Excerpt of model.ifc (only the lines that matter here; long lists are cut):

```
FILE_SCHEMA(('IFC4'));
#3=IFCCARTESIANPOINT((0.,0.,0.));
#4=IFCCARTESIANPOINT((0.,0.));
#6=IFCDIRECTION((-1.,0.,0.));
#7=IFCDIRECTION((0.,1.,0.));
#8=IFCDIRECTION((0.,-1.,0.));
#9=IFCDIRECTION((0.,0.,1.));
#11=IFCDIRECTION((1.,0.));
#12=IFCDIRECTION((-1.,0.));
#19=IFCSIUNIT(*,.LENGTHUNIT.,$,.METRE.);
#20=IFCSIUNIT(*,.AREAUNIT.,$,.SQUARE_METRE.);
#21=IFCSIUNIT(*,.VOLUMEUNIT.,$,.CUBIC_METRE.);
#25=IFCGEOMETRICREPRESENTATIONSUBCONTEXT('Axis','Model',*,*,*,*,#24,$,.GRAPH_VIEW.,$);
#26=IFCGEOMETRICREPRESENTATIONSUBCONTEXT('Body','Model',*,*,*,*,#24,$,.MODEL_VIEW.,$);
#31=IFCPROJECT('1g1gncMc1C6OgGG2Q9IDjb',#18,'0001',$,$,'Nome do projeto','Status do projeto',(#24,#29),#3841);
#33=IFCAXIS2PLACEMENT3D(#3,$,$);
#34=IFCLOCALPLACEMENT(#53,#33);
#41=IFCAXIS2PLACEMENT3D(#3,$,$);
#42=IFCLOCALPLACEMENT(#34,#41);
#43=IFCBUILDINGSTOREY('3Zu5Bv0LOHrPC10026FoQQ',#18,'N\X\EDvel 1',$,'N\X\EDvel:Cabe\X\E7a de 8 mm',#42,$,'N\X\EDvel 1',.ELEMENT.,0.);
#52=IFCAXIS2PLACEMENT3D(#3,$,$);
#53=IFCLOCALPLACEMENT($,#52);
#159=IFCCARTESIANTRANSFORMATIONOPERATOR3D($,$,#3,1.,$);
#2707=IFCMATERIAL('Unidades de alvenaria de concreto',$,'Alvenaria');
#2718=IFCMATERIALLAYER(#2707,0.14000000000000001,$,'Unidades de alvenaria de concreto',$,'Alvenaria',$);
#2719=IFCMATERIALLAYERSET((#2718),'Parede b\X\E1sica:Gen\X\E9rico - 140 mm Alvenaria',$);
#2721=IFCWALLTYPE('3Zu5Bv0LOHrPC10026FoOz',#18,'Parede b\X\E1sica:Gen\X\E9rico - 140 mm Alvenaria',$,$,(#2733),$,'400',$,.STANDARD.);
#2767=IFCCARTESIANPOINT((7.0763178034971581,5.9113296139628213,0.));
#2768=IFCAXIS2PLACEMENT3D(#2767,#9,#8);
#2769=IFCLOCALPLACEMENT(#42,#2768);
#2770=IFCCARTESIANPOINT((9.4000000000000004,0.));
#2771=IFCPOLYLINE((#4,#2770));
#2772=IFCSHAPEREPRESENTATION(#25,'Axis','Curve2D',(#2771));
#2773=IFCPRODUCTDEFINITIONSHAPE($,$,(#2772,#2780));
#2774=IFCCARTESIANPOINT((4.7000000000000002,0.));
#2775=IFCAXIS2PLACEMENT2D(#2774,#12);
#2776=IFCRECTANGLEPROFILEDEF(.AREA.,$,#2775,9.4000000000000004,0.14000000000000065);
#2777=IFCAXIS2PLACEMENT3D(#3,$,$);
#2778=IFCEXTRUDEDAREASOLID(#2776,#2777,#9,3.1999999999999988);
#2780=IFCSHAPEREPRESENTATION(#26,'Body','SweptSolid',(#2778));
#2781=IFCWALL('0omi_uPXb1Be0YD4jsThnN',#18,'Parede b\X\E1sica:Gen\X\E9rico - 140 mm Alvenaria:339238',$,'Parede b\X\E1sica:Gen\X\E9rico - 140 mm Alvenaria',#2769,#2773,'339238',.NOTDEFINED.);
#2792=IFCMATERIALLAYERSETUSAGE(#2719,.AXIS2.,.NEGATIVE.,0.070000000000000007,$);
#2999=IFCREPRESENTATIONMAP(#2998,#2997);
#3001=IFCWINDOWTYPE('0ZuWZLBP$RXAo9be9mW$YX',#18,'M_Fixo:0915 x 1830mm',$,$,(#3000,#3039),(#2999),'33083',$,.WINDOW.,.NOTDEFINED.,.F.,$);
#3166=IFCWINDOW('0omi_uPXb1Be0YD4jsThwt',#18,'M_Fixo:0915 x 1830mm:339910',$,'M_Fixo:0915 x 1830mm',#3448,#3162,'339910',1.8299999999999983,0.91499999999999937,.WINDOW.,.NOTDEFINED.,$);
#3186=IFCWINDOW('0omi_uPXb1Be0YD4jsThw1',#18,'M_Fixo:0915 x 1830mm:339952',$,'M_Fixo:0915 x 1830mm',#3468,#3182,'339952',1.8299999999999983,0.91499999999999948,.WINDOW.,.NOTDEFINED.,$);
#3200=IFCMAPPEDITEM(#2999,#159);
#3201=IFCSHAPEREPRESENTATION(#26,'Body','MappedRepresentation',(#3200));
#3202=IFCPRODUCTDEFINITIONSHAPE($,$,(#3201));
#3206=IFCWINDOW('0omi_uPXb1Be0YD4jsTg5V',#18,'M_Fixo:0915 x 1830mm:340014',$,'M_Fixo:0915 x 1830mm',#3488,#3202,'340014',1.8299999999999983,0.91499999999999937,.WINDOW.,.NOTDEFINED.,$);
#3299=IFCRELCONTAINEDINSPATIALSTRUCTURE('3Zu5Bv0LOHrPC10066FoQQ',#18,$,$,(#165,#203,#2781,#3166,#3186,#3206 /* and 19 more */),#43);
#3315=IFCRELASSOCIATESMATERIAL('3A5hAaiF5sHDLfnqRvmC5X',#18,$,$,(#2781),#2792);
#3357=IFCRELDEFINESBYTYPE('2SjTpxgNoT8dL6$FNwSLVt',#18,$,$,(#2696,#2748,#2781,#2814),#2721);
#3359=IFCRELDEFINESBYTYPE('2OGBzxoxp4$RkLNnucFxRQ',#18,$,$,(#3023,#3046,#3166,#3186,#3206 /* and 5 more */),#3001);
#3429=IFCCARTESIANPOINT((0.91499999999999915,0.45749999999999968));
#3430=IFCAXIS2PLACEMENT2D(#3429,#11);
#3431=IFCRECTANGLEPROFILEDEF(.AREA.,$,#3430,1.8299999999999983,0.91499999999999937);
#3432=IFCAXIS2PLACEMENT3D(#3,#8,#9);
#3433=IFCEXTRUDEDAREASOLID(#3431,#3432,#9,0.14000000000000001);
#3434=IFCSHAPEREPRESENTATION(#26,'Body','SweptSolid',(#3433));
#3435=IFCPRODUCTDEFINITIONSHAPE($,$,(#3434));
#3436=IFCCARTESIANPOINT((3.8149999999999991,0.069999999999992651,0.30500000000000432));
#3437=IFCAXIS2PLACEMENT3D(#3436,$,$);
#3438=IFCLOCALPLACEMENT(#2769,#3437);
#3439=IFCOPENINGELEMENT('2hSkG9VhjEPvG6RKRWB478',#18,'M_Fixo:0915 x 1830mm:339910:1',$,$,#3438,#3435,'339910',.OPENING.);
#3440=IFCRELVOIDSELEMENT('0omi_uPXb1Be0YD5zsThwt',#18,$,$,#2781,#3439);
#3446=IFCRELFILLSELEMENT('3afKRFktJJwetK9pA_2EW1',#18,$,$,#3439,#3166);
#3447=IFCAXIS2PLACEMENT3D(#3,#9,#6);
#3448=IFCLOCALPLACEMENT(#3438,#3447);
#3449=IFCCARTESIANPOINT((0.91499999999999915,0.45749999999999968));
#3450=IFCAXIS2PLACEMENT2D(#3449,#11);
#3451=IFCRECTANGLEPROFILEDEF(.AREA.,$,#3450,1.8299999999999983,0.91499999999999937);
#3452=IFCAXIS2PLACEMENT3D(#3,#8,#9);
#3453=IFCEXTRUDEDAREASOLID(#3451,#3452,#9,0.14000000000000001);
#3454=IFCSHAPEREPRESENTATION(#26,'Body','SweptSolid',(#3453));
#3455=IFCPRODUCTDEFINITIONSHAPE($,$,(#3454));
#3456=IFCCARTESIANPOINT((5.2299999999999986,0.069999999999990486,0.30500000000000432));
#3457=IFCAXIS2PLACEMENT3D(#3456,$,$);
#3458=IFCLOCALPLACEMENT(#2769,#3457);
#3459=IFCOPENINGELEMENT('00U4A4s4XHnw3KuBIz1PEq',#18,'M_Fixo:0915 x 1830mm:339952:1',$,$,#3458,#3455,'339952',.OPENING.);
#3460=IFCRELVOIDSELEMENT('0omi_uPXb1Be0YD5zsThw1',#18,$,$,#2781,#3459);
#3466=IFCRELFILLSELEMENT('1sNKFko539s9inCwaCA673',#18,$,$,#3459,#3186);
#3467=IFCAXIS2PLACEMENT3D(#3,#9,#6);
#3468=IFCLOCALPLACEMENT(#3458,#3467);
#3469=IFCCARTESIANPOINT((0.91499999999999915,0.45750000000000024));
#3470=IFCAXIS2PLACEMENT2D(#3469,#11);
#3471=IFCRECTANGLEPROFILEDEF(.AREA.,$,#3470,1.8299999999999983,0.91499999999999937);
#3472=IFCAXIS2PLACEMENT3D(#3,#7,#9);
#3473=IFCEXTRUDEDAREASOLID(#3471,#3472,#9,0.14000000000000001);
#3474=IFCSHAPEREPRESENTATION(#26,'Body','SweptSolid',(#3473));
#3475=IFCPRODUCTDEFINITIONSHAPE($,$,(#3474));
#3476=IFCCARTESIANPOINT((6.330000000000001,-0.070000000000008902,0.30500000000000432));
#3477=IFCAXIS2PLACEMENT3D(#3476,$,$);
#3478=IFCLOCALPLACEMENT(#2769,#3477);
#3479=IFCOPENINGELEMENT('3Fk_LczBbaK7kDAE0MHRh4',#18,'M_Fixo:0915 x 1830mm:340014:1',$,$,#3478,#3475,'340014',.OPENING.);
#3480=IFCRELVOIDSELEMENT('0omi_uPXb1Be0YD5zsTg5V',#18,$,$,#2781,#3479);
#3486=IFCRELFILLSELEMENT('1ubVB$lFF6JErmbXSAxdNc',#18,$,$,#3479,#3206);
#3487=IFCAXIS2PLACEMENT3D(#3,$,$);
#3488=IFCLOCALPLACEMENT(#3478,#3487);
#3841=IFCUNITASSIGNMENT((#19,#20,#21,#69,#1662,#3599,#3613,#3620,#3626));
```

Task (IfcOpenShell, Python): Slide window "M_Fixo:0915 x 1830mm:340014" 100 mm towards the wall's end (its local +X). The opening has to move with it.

```python
import ifcopenshell
import ifcopenshell.api.geometry
import ifcopenshell.util.placement
import ifcopenshell.util.unit

model = ifcopenshell.open("model.ifc")
unit_scale = ifcopenshell.util.unit.calculate_unit_scale(model)

window = model.by_guid("0omi_uPXb1Be0YD4jsTg5V")
opening = window.FillsVoids[0].RelatingOpeningElement
wall = opening.VoidsElements[0].RelatingBuildingElement

wall_matrix = ifcopenshell.util.placement.get_local_placement(wall.ObjectPlacement)
shift = wall_matrix[:3, 0] * 0.1 / unit_scale
before = ifcopenshell.util.placement.get_local_placement(window.ObjectPlacement)[:3, 3].copy()

# The window is placed relative to its opening, so it follows when the opening moves.
matrix = ifcopenshell.util.placement.get_local_placement(opening.ObjectPlacement)
matrix[:3, 3] += shift
ifcopenshell.api.geometry.edit_object_placement(
    model, product=opening, matrix=matrix, is_si=False, should_transform_children=True
)

after = ifcopenshell.util.placement.get_local_placement(window.ObjectPlacement)[:3, 3]
print("window moved by", (after - before).round(3) + 0.0)

model.write("model_edited.ifc")
```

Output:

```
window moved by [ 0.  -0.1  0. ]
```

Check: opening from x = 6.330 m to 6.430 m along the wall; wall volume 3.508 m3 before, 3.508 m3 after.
